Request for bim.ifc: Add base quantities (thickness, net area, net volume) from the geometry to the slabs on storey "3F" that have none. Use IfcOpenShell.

First a look at what the model holds.

```python
import ifcopenshell
import ifcopenshell.util.element
import ifcopenshell.util.unit

model = ifcopenshell.open("bim.ifc")
print(model.schema)
for unit_type in ("LENGTHUNIT", "AREAUNIT", "VOLUMEUNIT"):
    print(unit_type, ifcopenshell.util.unit.calculate_unit_scale(model, unit_type))
storey = next(s for s in model.by_type("IfcBuildingStorey") if s.Name == "3F")
slabs = [e for e in ifcopenshell.util.element.get_decomposition(storey) if e.is_a("IfcSlab")]
for e in sorted(slabs, key=lambda e: e.id()):
    print(e.id(), e.is_a(), e.Name, list(ifcopenshell.util.element.get_psets(e, qtos_only=True)), sep=" | ")
```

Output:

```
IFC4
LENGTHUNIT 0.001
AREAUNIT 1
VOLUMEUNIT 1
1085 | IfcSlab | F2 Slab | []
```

```python
import ifcopenshell
import ifcopenshell.api.pset
import ifcopenshell.geom
import ifcopenshell.util.element
import ifcopenshell.util.shape
import ifcopenshell.util.unit

model = ifcopenshell.open("bim.ifc")
unit_scale = ifcopenshell.util.unit.calculate_unit_scale(model)
area_scale = ifcopenshell.util.unit.calculate_unit_scale(model, "AREAUNIT")
volume_scale = ifcopenshell.util.unit.calculate_unit_scale(model, "VOLUMEUNIT")
settings = ifcopenshell.geom.settings()

storey = next(s for s in model.by_type("IfcBuildingStorey") if s.Name == "3F")
slabs = [e for e in ifcopenshell.util.element.get_decomposition(storey) if e.is_a("IfcSlab")]

for e in sorted(slabs, key=lambda e: e.id()):
    if ifcopenshell.util.element.get_psets(e, qtos_only=True, should_inherit=False):
        continue
    # Geometry comes back in metres, in the element's own axes.
    shape = ifcopenshell.geom.create_shape(settings, e)
    values = {
        "Width": ifcopenshell.util.shape.get_z(shape.geometry) / unit_scale,
        "NetArea": ifcopenshell.util.shape.get_footprint_area(shape.geometry) / area_scale,
        "NetVolume": ifcopenshell.util.shape.get_volume(shape.geometry) / volume_scale,
    }
    qto = ifcopenshell.api.pset.add_qto(model, product=e, name="Qto_SlabBaseQuantities")
    ifcopenshell.api.pset.edit_qto(model, qto=qto, properties=values)
    print(e.id(), {k: round(v, 3) for k, v in values.items()})

model.write("bim-out.ifc")
```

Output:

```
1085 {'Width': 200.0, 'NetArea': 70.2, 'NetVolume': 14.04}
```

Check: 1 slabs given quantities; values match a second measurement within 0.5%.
